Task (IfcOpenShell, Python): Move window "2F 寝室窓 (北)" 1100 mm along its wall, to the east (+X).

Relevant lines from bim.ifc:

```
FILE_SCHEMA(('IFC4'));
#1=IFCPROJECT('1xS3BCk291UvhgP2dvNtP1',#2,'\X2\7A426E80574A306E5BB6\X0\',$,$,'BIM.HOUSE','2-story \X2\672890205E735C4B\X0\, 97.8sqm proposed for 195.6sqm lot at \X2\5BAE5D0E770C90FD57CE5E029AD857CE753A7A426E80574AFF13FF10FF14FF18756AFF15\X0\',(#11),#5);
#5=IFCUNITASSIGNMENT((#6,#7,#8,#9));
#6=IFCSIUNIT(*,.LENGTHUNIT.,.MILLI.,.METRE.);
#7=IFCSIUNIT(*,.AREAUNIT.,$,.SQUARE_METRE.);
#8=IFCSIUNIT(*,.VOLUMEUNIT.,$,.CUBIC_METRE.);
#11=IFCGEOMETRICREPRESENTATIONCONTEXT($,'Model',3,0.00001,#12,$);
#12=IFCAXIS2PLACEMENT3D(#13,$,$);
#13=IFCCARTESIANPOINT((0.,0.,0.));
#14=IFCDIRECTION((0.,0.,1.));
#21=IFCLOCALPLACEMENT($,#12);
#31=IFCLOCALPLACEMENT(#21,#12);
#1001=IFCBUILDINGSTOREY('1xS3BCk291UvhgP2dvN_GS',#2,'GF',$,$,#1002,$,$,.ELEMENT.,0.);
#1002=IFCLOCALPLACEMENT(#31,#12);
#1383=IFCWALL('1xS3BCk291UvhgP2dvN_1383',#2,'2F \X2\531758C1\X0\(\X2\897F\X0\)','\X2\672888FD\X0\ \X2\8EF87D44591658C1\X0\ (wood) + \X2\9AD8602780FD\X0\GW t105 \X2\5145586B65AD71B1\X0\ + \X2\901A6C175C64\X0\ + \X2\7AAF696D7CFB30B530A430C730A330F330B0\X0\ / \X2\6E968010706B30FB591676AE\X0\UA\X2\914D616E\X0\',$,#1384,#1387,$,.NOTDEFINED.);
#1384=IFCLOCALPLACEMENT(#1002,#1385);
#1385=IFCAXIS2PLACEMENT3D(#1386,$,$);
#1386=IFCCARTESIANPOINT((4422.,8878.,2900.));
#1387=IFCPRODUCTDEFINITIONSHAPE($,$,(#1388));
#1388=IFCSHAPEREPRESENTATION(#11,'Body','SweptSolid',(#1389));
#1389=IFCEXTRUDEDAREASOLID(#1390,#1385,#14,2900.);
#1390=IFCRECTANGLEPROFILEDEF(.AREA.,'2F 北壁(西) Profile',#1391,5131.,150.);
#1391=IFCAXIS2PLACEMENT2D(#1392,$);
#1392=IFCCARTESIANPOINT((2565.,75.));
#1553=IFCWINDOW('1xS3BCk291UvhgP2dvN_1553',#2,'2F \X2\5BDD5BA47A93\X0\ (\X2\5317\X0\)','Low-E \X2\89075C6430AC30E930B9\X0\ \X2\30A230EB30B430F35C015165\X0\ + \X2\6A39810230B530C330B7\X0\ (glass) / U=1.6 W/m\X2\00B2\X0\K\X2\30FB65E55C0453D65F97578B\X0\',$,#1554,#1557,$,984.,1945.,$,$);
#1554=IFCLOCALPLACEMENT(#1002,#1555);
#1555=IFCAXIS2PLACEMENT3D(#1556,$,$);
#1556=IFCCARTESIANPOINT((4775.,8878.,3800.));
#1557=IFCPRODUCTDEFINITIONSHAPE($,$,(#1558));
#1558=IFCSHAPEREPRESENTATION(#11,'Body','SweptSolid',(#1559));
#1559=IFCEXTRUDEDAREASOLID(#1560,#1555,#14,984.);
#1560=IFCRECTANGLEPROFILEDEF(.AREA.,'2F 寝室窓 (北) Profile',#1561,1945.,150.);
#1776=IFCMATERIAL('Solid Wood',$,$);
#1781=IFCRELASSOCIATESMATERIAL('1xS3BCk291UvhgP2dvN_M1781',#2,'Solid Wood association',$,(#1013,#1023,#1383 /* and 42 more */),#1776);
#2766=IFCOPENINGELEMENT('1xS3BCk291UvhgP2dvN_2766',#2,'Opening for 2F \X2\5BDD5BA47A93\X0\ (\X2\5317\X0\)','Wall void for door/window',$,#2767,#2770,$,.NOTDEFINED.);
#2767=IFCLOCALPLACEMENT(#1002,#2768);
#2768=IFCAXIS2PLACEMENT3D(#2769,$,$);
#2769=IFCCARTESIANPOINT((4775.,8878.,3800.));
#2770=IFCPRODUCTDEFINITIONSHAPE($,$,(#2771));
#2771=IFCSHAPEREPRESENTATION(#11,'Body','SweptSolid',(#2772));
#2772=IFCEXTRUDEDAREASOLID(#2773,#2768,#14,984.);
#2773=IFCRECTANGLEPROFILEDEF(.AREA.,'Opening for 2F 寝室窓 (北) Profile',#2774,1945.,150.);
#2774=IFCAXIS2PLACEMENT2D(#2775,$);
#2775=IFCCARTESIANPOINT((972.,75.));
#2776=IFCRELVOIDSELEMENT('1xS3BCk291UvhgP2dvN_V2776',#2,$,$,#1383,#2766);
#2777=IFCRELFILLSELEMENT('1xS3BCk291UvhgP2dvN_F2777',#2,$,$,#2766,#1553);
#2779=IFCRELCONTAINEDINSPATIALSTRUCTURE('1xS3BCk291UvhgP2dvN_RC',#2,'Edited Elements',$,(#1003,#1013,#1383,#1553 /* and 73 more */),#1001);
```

```python
import ifcopenshell
import ifcopenshell.api.geometry
import ifcopenshell.util.placement
import ifcopenshell.util.unit

model = ifcopenshell.open("bim.ifc")
unit_scale = ifcopenshell.util.unit.calculate_unit_scale(model)

window = model.by_id(1553)
opening = window.FillsVoids[0].RelatingOpeningElement
wall = opening.VoidsElements[0].RelatingBuildingElement

wall_matrix = ifcopenshell.util.placement.get_local_placement(wall.ObjectPlacement)
shift = wall_matrix[:3, 0] * 1.1 / unit_scale
before = ifcopenshell.util.placement.get_local_placement(window.ObjectPlacement)[:3, 3].copy()

# The window is not placed relative to its opening, so move both.
for product in (opening, window):
    matrix = ifcopenshell.util.placement.get_local_placement(product.ObjectPlacement)
    matrix[:3, 3] += shift
    ifcopenshell.api.geometry.edit_object_placement(model, product=product, matrix=matrix, is_si=False)

after = ifcopenshell.util.placement.get_local_placement(window.ObjectPlacement)[:3, 3]
print("window moved by", (after - before).round(3) + 0.0)

model.write("bim-out.ifc")
```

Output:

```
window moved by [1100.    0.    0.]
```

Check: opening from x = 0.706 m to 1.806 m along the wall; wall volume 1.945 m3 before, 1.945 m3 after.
